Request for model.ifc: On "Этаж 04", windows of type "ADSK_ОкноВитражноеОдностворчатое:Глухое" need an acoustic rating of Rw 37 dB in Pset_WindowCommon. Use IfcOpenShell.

First a look at what the model holds.

```python
import ifcopenshell
import ifcopenshell.util.element

model = ifcopenshell.open("model.ifc")
print(model.schema)
storey = next(s for s in model.by_type("IfcBuildingStorey") if s.Name == "Этаж 04")
windows = [e for e in ifcopenshell.util.element.get_decomposition(storey) if e.is_a("IfcWindow")]
seen = {}
for e in windows:
    element_type = ifcopenshell.util.element.get_type(e)
    key = (element_type.Name if element_type != e and element_type else None, ifcopenshell.util.element.get_pset(e, "Pset_WindowCommon", "AcousticRating"))
    seen[key] = seen.get(key, 0) + 1
for (name, value), count in sorted(seen.items(), key=str):
    print(count, "x", name, "|", value)
```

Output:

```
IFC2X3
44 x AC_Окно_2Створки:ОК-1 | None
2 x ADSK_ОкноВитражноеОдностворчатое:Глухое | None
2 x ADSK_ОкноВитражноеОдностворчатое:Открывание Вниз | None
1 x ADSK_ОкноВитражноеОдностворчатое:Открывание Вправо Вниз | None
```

```python
import ifcopenshell
import ifcopenshell.api.pset
import ifcopenshell.util.element

model = ifcopenshell.open("model.ifc")

storey = next(s for s in model.by_type("IfcBuildingStorey") if s.Name == "Этаж 04")
windows = [e for e in ifcopenshell.util.element.get_decomposition(storey) if e.is_a("IfcWindow")]

count = 0
for e in windows:
    element_type = ifcopenshell.util.element.get_type(e)
    if element_type in (None, e) or element_type.Name != "ADSK_ОкноВитражноеОдностворчатое:Глухое":
        continue
    # add_pset returns the element's existing set when there is one.
    pset = ifcopenshell.api.pset.add_pset(model, product=e, name="Pset_WindowCommon")
    ifcopenshell.api.pset.edit_pset(model, pset=pset, properties={"AcousticRating": "Rw 37 dB"})
    count += 1

print(count, "windows updated")

model.write("model_edited.ifc")
```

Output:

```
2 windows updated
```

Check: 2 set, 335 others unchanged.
